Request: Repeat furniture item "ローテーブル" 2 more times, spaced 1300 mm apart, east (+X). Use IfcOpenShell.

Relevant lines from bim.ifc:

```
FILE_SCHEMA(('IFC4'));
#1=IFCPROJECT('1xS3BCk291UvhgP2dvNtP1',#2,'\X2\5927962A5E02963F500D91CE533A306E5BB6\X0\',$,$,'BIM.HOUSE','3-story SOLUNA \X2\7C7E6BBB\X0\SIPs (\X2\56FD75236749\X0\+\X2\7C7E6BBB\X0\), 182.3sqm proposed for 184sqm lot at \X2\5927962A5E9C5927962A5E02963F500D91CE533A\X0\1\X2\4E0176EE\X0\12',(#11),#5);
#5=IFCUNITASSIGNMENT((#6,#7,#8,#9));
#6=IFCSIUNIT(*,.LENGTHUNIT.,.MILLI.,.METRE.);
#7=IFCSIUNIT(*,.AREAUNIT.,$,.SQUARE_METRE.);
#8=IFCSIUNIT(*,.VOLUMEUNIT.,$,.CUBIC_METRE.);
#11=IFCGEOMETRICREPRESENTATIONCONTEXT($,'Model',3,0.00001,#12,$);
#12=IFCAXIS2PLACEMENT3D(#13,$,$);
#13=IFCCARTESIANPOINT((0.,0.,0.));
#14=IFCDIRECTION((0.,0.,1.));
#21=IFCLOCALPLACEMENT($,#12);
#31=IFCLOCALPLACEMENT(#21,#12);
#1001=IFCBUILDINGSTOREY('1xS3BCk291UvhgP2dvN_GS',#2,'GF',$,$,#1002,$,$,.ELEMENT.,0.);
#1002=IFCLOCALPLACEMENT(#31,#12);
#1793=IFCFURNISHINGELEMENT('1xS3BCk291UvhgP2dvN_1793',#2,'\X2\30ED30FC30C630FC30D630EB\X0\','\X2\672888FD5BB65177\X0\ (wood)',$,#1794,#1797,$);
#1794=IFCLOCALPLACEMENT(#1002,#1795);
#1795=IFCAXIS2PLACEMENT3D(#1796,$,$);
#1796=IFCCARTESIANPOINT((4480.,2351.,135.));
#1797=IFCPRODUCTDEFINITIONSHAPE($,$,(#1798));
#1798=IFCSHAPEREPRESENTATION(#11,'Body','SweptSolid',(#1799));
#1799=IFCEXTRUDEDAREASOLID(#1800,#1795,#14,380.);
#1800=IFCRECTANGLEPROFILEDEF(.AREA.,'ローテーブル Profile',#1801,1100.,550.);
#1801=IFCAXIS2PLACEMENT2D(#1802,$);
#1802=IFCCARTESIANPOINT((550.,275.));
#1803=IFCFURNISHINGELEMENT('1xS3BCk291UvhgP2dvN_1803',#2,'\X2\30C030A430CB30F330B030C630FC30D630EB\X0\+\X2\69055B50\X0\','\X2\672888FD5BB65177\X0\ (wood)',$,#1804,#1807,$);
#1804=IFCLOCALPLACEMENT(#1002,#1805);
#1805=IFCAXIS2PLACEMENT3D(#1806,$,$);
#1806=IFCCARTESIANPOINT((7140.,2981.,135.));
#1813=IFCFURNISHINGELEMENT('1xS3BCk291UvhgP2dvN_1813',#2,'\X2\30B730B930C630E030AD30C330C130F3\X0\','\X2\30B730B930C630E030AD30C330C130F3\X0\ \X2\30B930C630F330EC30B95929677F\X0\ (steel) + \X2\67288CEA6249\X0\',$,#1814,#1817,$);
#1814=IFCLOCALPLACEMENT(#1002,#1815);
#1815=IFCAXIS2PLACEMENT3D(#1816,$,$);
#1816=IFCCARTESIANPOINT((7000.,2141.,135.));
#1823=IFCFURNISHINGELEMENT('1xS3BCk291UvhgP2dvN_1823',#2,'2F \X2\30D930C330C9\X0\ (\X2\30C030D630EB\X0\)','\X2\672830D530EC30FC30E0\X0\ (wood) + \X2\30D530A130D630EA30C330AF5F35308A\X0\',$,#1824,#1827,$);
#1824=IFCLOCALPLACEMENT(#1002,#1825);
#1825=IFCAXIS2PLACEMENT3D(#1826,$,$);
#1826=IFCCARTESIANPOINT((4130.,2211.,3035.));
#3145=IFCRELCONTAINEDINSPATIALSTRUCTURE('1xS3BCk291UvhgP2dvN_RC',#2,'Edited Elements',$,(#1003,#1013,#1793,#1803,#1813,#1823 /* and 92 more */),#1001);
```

```python
import numpy as np
import ifcopenshell
import ifcopenshell.api.geometry
import ifcopenshell.api.root
import ifcopenshell.util.element
import ifcopenshell.util.placement
import ifcopenshell.util.unit

model = ifcopenshell.open("bim.ifc")
unit_scale = ifcopenshell.util.unit.calculate_unit_scale(model)


def reuse_history(source, copy):
    """copy_class also copies each property set's owner history, people and application; keep the originals."""
    for rel in copy.IsDefinedBy:
        if rel.is_a("IfcRelDefinesByProperties") and (history := rel.RelatingPropertyDefinition.OwnerHistory):
            rel.RelatingPropertyDefinition.OwnerHistory = source.OwnerHistory
            ifcopenshell.util.element.remove_deep2(model, history)


source = model.by_id(1793)
base = ifcopenshell.util.placement.get_local_placement(source.ObjectPlacement)
step = np.array([1.0, 0.0, 0.0]) * 1.3 / unit_scale

for i in range(1, 3):
    copy = ifcopenshell.api.root.copy_class(model, product=source)
    copy.Representation = ifcopenshell.util.element.copy_deep(
        model, source.Representation, exclude=["IfcGeometricRepresentationContext", "IfcRepresentationMap"]
    )
    reuse_history(source, copy)
    matrix = base.copy()
    matrix[:3, 3] += i * step
    print("added at", matrix[:3, 3].round(3) + 0.0)
    ifcopenshell.api.geometry.edit_object_placement(model, product=copy, matrix=matrix, is_si=False)

model.write("bim-out.ifc")
```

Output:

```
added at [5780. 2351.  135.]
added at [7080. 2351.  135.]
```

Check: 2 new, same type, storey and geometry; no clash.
